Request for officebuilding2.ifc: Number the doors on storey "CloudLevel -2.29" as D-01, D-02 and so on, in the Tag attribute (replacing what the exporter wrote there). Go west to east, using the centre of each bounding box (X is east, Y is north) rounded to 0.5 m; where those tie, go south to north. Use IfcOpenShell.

First a look at what the model holds.

```python
import ifcopenshell
import ifcopenshell.util.element
import ifcopenshell.util.placement

model = ifcopenshell.open("officebuilding2.ifc")
print(model.schema)
storey = next(s for s in model.by_type("IfcBuildingStorey") if s.Name == "CloudLevel -2.29")
doors = [e for e in ifcopenshell.util.element.get_decomposition(storey) if e.is_a("IfcDoor")]
for e in sorted(doors, key=lambda e: e.id()):
    origin = ifcopenshell.util.placement.get_local_placement(e.ObjectPlacement)[:3, 3]
    print(e.id(), e.Tag, e.Name, origin.round(2) + 0.0, sep=" | ")
```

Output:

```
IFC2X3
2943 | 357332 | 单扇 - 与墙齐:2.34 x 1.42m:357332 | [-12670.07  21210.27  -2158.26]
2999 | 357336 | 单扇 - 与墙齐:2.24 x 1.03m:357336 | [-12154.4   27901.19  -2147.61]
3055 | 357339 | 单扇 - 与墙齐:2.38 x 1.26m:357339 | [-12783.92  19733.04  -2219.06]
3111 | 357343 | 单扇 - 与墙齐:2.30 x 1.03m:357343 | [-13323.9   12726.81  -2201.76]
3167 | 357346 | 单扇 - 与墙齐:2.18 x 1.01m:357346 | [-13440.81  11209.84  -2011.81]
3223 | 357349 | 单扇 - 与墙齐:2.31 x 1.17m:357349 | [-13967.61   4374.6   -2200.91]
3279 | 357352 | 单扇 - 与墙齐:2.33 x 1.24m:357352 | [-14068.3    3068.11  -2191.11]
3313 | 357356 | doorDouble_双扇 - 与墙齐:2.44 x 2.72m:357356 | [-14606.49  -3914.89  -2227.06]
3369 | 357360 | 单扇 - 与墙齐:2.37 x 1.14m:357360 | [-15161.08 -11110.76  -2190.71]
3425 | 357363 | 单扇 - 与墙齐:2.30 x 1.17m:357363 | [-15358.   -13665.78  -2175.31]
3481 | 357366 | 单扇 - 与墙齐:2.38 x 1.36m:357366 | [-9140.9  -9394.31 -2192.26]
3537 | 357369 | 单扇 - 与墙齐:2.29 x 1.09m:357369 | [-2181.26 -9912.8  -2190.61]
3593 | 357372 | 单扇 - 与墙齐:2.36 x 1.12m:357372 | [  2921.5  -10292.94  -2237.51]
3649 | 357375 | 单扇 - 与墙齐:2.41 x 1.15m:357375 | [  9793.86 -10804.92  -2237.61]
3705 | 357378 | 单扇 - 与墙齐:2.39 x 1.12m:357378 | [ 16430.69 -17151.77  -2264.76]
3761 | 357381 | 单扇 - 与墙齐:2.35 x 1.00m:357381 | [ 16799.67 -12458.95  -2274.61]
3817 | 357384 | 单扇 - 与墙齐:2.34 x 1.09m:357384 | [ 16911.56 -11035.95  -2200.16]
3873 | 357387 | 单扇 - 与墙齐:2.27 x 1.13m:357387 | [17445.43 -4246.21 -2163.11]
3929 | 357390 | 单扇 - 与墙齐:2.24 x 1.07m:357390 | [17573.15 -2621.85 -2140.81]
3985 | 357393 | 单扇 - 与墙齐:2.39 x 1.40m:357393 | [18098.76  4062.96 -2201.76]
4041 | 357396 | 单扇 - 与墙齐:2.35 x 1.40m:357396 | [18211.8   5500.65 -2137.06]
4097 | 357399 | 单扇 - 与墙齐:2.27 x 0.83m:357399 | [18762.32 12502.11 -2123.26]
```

```python
import ifcopenshell
import ifcopenshell.geom
import ifcopenshell.util.element
import ifcopenshell.util.shape

model = ifcopenshell.open("officebuilding2.ifc")
settings = ifcopenshell.geom.settings()
settings.set("use-world-coords", True)


def centre(element):
    shape = ifcopenshell.geom.create_shape(settings, element)
    return ifcopenshell.util.shape.get_bbox_centroid(shape.geometry)


storey = next(s for s in model.by_type("IfcBuildingStorey") if s.Name == "CloudLevel -2.29")
doors = [e for e in ifcopenshell.util.element.get_decomposition(storey) if e.is_a("IfcDoor")]

# Insertion points can sit at a corner or the storey origin, so sort by the geometry (in metres).
centres = {e: centre(e) for e in doors}
doors.sort(key=lambda e: (round(centres[e][0] / 0.5), centres[e][1]))

for i, e in enumerate(doors, start=1):
    number = f"D-{i:02d}"
    e.Tag = number
    print(e.id(), number)

model.write("officebuilding2_rev.ifc")
```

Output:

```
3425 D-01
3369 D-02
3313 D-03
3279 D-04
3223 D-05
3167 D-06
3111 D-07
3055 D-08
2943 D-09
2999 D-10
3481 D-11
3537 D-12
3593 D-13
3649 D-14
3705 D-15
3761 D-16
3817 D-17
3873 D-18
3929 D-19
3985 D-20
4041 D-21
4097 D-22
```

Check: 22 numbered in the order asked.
